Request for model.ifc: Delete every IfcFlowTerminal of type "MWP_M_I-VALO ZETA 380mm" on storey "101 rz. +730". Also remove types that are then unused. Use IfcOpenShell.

First a look at what the model holds.

```python
import ifcopenshell
import ifcopenshell.util.element

model = ifcopenshell.open("model.ifc")
print(model.schema)
storey = next(s for s in model.by_type("IfcBuildingStorey") if s.Name == "101 rz. +730")
terminals = [e for e in ifcopenshell.util.element.get_decomposition(storey) if e.is_a("IfcFlowTerminal")]
seen = {}
for e in terminals:
    element_type = ifcopenshell.util.element.get_type(e)
    name = element_type.Name if element_type not in (None, e) else None
    seen[name] = seen.get(name, 0) + 1
for name, count in sorted(seen.items(), key=str):
    print(count, "x", name)
```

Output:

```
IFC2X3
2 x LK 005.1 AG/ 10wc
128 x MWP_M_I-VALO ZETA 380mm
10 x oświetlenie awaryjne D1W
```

```python
import ifcopenshell
import ifcopenshell.api.root
import ifcopenshell.util.element

model = ifcopenshell.open("model.ifc")

storey = next(s for s in model.by_type("IfcBuildingStorey") if s.Name == "101 rz. +730")
terminals = [e for e in ifcopenshell.util.element.get_decomposition(storey) if e.is_a("IfcFlowTerminal")]
targets = [e for e in terminals if (t := ifcopenshell.util.element.get_type(e)) not in (None, e) and t.Name == "MWP_M_I-VALO ZETA 380mm"]
types = {ifcopenshell.util.element.get_type(e) for e in targets} - {None, *targets}

for e in targets:
    ifcopenshell.api.root.remove_product(model, product=e)
print(len(targets), "removed")

unused = [t for t in types if not ifcopenshell.util.element.get_types(t)]
for t in unused:
    ifcopenshell.api.root.remove_product(model, product=t)
print(len(unused), "unused types removed")

model.write("model_rev.ifc")
```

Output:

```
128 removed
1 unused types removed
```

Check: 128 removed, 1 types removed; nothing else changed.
